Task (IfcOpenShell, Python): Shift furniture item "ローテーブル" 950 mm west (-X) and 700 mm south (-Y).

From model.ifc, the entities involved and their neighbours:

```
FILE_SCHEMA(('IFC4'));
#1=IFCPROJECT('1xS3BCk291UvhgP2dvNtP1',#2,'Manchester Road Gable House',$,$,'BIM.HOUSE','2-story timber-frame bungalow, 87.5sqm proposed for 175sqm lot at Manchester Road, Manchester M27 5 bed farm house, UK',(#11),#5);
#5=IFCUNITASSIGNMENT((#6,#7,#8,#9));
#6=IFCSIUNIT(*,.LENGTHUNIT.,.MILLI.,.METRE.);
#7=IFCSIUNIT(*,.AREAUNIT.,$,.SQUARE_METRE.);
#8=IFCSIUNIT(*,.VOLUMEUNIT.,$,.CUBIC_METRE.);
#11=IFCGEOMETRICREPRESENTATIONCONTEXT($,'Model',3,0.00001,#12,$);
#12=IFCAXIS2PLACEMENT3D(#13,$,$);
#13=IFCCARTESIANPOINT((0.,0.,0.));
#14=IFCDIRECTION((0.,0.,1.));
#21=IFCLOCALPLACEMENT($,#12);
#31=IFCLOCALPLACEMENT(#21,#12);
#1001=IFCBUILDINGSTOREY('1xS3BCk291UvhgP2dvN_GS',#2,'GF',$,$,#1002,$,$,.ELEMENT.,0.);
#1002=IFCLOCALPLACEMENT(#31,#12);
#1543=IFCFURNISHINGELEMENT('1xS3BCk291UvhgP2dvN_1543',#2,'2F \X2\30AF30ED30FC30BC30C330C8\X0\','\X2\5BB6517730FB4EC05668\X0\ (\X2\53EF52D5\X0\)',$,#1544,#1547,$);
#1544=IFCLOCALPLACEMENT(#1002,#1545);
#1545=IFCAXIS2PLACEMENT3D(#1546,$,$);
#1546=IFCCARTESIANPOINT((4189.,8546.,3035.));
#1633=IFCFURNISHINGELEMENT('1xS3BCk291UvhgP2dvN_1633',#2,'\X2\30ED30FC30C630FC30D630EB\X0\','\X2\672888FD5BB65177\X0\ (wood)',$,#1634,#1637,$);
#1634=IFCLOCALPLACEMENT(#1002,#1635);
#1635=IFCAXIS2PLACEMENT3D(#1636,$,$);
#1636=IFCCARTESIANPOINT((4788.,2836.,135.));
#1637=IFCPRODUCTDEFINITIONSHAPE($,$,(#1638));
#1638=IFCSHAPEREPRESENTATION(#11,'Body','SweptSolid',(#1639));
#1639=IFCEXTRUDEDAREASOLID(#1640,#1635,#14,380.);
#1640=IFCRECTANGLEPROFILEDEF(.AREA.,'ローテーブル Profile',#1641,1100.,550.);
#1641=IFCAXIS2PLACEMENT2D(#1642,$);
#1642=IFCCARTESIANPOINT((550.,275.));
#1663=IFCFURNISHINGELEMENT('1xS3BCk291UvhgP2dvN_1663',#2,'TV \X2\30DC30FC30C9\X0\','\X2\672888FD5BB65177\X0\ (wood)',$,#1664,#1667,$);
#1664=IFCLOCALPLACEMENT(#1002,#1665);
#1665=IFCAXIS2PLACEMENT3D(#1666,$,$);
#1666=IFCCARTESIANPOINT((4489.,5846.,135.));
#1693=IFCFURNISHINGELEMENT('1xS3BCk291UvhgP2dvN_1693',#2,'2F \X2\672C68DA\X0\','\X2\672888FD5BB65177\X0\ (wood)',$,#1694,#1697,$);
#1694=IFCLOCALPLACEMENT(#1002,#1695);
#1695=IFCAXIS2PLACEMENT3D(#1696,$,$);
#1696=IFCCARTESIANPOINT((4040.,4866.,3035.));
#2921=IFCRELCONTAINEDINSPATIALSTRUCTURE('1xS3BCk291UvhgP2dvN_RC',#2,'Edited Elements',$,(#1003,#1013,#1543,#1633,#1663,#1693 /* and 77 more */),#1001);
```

```python
import ifcopenshell
import ifcopenshell.api.geometry
import ifcopenshell.util.placement
import ifcopenshell.util.unit

model = ifcopenshell.open("model.ifc")
unit_scale = ifcopenshell.util.unit.calculate_unit_scale(model)

item = model.by_guid("1xS3BCk291UvhgP2dvN_1633")
matrix = ifcopenshell.util.placement.get_local_placement(item.ObjectPlacement)
matrix[0, 3] -= 0.95 / unit_scale
matrix[1, 3] -= 0.7 / unit_scale
ifcopenshell.api.geometry.edit_object_placement(model, product=item, matrix=matrix, is_si=False)

print(ifcopenshell.util.placement.get_local_placement(item.ObjectPlacement).round(3) + 0.0)

model.write("model_updated.ifc")
```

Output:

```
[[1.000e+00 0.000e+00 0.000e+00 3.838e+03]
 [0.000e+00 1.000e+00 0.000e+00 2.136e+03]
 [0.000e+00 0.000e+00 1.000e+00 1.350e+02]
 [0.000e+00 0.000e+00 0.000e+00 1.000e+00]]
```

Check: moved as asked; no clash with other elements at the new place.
